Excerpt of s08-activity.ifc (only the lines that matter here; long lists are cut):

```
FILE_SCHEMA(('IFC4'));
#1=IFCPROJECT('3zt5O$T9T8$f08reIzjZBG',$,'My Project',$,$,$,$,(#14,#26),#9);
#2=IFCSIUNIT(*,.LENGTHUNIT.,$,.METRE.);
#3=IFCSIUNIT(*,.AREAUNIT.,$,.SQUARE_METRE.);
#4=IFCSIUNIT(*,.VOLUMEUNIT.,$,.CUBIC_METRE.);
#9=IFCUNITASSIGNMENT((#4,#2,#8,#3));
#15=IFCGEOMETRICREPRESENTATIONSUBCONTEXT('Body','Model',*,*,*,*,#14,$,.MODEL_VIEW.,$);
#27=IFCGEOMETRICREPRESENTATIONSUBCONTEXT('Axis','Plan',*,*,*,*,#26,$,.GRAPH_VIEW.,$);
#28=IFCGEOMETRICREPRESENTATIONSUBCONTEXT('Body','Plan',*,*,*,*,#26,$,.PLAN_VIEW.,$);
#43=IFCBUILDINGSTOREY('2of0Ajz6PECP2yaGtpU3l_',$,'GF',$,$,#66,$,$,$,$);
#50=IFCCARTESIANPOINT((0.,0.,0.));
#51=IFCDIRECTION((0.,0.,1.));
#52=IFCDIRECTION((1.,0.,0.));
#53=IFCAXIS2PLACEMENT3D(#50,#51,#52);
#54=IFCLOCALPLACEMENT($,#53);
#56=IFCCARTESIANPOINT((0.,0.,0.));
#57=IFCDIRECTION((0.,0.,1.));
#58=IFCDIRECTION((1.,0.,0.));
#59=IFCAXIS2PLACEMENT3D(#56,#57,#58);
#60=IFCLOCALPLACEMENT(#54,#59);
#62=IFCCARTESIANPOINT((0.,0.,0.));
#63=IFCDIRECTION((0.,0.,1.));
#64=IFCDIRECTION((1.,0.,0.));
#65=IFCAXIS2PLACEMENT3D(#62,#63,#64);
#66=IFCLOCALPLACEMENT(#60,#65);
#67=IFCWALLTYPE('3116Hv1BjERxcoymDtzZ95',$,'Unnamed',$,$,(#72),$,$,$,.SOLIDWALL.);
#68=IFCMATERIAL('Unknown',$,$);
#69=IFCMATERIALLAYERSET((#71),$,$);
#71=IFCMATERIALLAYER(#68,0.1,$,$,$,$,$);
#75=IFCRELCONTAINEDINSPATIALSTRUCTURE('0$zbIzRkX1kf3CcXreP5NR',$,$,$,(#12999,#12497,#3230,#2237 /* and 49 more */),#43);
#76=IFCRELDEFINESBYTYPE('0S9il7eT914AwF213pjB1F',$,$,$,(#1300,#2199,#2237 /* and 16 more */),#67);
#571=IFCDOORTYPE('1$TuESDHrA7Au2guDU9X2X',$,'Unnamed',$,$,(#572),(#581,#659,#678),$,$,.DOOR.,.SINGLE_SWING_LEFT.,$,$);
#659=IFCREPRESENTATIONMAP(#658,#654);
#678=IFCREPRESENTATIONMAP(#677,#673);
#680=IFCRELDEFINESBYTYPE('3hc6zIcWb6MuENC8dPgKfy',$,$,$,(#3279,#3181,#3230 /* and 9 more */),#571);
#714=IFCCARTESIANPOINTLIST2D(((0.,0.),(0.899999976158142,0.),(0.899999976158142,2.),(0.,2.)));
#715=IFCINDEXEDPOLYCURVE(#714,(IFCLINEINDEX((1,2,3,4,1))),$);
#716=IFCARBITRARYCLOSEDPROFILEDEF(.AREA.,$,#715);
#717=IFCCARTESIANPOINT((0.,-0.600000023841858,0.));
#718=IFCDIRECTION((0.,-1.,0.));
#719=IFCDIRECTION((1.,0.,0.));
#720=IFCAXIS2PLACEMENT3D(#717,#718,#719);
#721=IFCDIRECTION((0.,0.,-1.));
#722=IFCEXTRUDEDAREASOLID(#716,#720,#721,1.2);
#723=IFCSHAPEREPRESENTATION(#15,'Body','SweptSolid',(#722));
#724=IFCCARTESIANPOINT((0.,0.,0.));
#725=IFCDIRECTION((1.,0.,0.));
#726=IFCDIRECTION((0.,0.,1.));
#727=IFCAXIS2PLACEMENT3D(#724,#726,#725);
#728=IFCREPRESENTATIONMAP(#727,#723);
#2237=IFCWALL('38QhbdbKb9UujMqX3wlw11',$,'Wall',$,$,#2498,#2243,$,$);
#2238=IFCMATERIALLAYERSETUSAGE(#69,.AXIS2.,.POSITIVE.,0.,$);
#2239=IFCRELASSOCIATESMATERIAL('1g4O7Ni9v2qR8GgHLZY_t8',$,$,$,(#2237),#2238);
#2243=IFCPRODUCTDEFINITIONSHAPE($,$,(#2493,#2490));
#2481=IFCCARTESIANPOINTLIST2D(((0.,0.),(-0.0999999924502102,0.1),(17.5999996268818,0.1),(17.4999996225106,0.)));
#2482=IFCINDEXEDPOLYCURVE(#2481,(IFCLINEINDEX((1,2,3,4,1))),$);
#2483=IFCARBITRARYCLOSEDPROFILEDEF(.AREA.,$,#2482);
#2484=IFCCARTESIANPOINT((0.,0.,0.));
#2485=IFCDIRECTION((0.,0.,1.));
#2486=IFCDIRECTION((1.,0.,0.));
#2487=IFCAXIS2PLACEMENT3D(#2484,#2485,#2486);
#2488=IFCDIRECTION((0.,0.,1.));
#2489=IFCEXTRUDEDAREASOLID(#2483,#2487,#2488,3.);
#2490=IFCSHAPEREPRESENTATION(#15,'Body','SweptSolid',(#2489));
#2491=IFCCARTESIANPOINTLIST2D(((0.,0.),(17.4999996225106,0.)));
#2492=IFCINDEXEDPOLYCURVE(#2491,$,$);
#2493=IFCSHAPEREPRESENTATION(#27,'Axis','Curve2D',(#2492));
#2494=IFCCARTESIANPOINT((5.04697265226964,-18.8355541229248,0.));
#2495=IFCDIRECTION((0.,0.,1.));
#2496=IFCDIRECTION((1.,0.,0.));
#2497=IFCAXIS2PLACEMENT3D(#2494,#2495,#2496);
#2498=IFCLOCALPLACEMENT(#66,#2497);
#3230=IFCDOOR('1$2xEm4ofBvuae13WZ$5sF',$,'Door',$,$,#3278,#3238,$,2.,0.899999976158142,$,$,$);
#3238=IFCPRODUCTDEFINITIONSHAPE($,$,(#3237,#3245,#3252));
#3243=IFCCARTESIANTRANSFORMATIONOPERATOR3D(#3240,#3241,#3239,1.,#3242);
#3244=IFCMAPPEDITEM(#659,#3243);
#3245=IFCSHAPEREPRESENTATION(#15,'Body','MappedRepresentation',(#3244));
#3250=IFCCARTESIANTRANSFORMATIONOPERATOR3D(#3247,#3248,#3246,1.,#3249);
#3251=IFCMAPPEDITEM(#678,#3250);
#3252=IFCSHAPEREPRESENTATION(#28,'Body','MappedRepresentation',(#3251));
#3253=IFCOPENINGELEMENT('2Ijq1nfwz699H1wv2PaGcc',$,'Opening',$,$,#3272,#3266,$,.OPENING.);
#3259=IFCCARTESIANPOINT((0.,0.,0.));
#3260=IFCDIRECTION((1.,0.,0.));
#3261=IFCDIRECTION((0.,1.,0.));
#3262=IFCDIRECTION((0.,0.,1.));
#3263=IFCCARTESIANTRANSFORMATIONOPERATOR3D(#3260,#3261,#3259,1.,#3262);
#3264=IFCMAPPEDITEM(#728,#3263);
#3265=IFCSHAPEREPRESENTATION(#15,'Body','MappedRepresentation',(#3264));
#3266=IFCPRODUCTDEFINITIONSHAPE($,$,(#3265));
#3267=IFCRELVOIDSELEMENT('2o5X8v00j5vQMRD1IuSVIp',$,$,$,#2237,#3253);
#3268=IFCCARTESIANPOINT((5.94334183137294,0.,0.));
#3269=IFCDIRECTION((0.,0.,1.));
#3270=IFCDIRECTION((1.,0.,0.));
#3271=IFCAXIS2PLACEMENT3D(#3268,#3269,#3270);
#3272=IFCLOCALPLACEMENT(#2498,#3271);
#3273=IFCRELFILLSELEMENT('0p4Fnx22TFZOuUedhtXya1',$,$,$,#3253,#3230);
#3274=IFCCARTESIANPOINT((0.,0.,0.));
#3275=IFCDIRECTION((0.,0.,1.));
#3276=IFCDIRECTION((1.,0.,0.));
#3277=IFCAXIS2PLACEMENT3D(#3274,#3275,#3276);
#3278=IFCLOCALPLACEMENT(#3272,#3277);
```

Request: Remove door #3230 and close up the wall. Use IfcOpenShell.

```python
import ifcopenshell
import ifcopenshell.api.feature
import ifcopenshell.api.root
import ifcopenshell.geom
import ifcopenshell.util.shape

model = ifcopenshell.open("s08-activity.ifc")
settings = ifcopenshell.geom.settings()


def volume(element):
    """Net volume in cubic metres, openings subtracted."""
    shape = ifcopenshell.geom.create_shape(settings, element)
    return ifcopenshell.util.shape.get_volume(shape.geometry)


door = model.by_guid("1$2xEm4ofBvuae13WZ$5sF")
opening = door.FillsVoids[0].RelatingOpeningElement
wall = opening.VoidsElements[0].RelatingBuildingElement
before = volume(wall)

ifcopenshell.api.root.remove_product(model, product=door)
ifcopenshell.api.feature.remove_feature(model, feature=opening)

after = volume(wall)

print(f"wall volume {before:.3f} -> {after:.3f} m3")

model.write("s08-activity-out.ifc")
```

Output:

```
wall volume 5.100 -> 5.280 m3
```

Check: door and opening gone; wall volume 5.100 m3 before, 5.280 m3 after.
